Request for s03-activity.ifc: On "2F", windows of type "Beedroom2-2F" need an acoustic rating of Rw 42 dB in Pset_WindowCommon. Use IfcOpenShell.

First a look at what the model holds.

```python
import ifcopenshell
import ifcopenshell.util.element

model = ifcopenshell.open("s03-activity.ifc")
print(model.schema)
storey = next(s for s in model.by_type("IfcBuildingStorey") if s.Name == "2F")
windows = [e for e in ifcopenshell.util.element.get_decomposition(storey) if e.is_a("IfcWindow")]
seen = {}
for e in windows:
    element_type = ifcopenshell.util.element.get_type(e)
    key = (element_type.Name if element_type != e and element_type else None, ifcopenshell.util.element.get_pset(e, "Pset_WindowCommon", "AcousticRating"))
    seen[key] = seen.get(key, 0) + 1
for (name, value), count in sorted(seen.items(), key=str):
    print(count, "x", name, "|", value)
```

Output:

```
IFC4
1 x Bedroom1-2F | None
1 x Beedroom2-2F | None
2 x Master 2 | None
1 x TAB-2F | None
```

```python
import ifcopenshell
import ifcopenshell.api.pset
import ifcopenshell.util.element

model = ifcopenshell.open("s03-activity.ifc")

storey = next(s for s in model.by_type("IfcBuildingStorey") if s.Name == "2F")
windows = [e for e in ifcopenshell.util.element.get_decomposition(storey) if e.is_a("IfcWindow")]

count = 0
for e in windows:
    element_type = ifcopenshell.util.element.get_type(e)
    if element_type in (None, e) or element_type.Name != "Beedroom2-2F":
        continue
    # add_pset returns the element's existing set when there is one.
    pset = ifcopenshell.api.pset.add_pset(model, product=e, name="Pset_WindowCommon")
    ifcopenshell.api.pset.edit_pset(model, pset=pset, properties={"AcousticRating": "Rw 42 dB"})
    count += 1

print(count, "windows updated")

model.write("s03-activity_edited.ifc")
```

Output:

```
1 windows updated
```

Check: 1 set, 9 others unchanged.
